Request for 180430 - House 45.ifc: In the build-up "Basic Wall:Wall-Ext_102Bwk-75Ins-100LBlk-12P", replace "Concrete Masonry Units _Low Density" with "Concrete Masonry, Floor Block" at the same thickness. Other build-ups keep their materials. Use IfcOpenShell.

First a look at what the model holds.

```python
import ifcopenshell
import ifcopenshell.util.element

model = ifcopenshell.open("180430 - House 45.ifc")
print(model.schema)
for layer_set in model.by_type("IfcMaterialLayerSet"):
    if layer_set.LayerSetName == "Basic Wall:Wall-Ext_102Bwk-75Ins-100LBlk-12P":
        for layer in layer_set.MaterialLayers:
            print(layer.id(), layer.Material and layer.Material.Name, layer.LayerThickness, sep=" | ")
        print(len(ifcopenshell.util.element.get_elements_by_material(model, layer_set)), "elements and types use it")
print(sorted(m.Name for m in model.by_type("IfcMaterial") if m.Name)[:60])
```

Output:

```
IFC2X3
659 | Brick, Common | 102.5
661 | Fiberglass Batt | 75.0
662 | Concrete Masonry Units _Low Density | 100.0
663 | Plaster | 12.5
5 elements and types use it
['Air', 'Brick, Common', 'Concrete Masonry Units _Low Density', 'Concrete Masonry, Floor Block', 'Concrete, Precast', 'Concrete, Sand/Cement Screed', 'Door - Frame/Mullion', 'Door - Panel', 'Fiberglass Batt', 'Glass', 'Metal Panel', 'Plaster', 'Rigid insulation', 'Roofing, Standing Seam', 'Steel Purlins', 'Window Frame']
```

```python
import ifcopenshell
import ifcopenshell.api.material

model = ifcopenshell.open("180430 - House 45.ifc")

layer_set = next(s for s in model.by_type("IfcMaterialLayerSet") if s.LayerSetName == "Basic Wall:Wall-Ext_102Bwk-75Ins-100LBlk-12P")
layer = next(l for l in layer_set.MaterialLayers if l.Material and l.Material.Name == "Concrete Masonry Units _Low Density")
material = next(m for m in model.by_type("IfcMaterial") if m.Name == "Concrete Masonry, Floor Block")

# Point this one layer at the other material; renaming the old one would change it everywhere.
ifcopenshell.api.material.edit_layer(model, layer=layer, attributes={}, material=material)

print([l.Material.Name if l.Material else None for l in layer_set.MaterialLayers])

model.write("180430 - House 45_v2.ifc")
```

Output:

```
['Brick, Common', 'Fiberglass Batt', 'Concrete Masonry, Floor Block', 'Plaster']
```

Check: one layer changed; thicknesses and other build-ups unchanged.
